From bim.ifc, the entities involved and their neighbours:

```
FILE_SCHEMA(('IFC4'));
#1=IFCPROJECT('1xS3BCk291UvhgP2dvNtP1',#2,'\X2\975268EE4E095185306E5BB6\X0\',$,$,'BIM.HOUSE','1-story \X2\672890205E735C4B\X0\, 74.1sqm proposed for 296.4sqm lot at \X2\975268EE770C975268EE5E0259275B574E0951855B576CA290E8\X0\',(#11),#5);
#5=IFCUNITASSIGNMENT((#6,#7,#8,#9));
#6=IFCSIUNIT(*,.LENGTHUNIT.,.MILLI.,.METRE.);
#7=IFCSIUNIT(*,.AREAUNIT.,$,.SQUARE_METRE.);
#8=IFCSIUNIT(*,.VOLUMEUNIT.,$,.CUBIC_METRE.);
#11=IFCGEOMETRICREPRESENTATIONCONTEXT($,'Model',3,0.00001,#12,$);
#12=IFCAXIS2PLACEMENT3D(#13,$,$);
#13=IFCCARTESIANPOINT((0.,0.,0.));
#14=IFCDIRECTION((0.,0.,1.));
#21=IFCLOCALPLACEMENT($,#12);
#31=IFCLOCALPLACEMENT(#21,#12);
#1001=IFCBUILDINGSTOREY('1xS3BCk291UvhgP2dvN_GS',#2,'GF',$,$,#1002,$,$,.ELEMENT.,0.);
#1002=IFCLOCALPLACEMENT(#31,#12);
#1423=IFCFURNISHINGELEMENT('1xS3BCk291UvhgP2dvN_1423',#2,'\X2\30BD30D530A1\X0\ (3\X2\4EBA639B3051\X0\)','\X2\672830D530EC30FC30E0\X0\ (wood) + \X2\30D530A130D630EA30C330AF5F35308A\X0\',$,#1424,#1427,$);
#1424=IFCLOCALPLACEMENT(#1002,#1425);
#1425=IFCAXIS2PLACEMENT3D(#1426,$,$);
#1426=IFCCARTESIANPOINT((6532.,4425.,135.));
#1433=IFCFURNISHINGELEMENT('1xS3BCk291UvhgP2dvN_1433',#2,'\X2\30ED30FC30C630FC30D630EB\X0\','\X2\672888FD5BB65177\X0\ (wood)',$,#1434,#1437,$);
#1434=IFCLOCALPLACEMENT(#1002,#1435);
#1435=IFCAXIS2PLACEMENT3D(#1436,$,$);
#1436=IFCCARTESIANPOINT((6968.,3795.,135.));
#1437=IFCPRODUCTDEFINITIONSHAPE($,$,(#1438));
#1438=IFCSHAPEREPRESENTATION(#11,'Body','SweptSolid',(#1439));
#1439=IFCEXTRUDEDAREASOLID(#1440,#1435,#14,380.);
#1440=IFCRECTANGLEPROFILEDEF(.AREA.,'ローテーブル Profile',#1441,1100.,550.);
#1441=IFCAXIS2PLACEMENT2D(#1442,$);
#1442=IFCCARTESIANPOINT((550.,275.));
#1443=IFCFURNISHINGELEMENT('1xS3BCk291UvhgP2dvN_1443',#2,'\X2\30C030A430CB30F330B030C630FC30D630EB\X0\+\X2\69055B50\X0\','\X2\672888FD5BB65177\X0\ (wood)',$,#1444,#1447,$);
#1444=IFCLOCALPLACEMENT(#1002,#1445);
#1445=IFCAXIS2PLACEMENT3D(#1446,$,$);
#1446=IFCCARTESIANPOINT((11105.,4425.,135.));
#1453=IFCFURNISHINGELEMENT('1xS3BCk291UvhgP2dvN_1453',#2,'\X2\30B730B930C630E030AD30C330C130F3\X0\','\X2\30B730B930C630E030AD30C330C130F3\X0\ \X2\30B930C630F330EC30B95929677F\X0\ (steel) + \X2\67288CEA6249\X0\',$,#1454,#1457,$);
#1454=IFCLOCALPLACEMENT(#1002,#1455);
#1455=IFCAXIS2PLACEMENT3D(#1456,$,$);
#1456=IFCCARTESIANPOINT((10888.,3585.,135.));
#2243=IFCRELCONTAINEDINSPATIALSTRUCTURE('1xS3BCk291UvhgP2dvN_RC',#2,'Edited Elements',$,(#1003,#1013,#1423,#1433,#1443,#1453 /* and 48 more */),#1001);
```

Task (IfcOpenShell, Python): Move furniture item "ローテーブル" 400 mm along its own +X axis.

```python
import ifcopenshell
import ifcopenshell.api.geometry
import ifcopenshell.util.placement
import ifcopenshell.util.unit

model = ifcopenshell.open("bim.ifc")
unit_scale = ifcopenshell.util.unit.calculate_unit_scale(model)

item = model.by_id(1433)
matrix = ifcopenshell.util.placement.get_local_placement(item.ObjectPlacement)
matrix[:3, 3] += matrix[:3, 0] * 0.4 / unit_scale
ifcopenshell.api.geometry.edit_object_placement(model, product=item, matrix=matrix, is_si=False)

print(ifcopenshell.util.placement.get_local_placement(item.ObjectPlacement).round(3) + 0.0)

model.write("bim_updated.ifc")
```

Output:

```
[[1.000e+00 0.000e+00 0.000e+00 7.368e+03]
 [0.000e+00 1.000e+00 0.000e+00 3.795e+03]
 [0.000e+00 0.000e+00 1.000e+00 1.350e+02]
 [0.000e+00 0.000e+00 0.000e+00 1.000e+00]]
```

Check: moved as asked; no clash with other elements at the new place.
